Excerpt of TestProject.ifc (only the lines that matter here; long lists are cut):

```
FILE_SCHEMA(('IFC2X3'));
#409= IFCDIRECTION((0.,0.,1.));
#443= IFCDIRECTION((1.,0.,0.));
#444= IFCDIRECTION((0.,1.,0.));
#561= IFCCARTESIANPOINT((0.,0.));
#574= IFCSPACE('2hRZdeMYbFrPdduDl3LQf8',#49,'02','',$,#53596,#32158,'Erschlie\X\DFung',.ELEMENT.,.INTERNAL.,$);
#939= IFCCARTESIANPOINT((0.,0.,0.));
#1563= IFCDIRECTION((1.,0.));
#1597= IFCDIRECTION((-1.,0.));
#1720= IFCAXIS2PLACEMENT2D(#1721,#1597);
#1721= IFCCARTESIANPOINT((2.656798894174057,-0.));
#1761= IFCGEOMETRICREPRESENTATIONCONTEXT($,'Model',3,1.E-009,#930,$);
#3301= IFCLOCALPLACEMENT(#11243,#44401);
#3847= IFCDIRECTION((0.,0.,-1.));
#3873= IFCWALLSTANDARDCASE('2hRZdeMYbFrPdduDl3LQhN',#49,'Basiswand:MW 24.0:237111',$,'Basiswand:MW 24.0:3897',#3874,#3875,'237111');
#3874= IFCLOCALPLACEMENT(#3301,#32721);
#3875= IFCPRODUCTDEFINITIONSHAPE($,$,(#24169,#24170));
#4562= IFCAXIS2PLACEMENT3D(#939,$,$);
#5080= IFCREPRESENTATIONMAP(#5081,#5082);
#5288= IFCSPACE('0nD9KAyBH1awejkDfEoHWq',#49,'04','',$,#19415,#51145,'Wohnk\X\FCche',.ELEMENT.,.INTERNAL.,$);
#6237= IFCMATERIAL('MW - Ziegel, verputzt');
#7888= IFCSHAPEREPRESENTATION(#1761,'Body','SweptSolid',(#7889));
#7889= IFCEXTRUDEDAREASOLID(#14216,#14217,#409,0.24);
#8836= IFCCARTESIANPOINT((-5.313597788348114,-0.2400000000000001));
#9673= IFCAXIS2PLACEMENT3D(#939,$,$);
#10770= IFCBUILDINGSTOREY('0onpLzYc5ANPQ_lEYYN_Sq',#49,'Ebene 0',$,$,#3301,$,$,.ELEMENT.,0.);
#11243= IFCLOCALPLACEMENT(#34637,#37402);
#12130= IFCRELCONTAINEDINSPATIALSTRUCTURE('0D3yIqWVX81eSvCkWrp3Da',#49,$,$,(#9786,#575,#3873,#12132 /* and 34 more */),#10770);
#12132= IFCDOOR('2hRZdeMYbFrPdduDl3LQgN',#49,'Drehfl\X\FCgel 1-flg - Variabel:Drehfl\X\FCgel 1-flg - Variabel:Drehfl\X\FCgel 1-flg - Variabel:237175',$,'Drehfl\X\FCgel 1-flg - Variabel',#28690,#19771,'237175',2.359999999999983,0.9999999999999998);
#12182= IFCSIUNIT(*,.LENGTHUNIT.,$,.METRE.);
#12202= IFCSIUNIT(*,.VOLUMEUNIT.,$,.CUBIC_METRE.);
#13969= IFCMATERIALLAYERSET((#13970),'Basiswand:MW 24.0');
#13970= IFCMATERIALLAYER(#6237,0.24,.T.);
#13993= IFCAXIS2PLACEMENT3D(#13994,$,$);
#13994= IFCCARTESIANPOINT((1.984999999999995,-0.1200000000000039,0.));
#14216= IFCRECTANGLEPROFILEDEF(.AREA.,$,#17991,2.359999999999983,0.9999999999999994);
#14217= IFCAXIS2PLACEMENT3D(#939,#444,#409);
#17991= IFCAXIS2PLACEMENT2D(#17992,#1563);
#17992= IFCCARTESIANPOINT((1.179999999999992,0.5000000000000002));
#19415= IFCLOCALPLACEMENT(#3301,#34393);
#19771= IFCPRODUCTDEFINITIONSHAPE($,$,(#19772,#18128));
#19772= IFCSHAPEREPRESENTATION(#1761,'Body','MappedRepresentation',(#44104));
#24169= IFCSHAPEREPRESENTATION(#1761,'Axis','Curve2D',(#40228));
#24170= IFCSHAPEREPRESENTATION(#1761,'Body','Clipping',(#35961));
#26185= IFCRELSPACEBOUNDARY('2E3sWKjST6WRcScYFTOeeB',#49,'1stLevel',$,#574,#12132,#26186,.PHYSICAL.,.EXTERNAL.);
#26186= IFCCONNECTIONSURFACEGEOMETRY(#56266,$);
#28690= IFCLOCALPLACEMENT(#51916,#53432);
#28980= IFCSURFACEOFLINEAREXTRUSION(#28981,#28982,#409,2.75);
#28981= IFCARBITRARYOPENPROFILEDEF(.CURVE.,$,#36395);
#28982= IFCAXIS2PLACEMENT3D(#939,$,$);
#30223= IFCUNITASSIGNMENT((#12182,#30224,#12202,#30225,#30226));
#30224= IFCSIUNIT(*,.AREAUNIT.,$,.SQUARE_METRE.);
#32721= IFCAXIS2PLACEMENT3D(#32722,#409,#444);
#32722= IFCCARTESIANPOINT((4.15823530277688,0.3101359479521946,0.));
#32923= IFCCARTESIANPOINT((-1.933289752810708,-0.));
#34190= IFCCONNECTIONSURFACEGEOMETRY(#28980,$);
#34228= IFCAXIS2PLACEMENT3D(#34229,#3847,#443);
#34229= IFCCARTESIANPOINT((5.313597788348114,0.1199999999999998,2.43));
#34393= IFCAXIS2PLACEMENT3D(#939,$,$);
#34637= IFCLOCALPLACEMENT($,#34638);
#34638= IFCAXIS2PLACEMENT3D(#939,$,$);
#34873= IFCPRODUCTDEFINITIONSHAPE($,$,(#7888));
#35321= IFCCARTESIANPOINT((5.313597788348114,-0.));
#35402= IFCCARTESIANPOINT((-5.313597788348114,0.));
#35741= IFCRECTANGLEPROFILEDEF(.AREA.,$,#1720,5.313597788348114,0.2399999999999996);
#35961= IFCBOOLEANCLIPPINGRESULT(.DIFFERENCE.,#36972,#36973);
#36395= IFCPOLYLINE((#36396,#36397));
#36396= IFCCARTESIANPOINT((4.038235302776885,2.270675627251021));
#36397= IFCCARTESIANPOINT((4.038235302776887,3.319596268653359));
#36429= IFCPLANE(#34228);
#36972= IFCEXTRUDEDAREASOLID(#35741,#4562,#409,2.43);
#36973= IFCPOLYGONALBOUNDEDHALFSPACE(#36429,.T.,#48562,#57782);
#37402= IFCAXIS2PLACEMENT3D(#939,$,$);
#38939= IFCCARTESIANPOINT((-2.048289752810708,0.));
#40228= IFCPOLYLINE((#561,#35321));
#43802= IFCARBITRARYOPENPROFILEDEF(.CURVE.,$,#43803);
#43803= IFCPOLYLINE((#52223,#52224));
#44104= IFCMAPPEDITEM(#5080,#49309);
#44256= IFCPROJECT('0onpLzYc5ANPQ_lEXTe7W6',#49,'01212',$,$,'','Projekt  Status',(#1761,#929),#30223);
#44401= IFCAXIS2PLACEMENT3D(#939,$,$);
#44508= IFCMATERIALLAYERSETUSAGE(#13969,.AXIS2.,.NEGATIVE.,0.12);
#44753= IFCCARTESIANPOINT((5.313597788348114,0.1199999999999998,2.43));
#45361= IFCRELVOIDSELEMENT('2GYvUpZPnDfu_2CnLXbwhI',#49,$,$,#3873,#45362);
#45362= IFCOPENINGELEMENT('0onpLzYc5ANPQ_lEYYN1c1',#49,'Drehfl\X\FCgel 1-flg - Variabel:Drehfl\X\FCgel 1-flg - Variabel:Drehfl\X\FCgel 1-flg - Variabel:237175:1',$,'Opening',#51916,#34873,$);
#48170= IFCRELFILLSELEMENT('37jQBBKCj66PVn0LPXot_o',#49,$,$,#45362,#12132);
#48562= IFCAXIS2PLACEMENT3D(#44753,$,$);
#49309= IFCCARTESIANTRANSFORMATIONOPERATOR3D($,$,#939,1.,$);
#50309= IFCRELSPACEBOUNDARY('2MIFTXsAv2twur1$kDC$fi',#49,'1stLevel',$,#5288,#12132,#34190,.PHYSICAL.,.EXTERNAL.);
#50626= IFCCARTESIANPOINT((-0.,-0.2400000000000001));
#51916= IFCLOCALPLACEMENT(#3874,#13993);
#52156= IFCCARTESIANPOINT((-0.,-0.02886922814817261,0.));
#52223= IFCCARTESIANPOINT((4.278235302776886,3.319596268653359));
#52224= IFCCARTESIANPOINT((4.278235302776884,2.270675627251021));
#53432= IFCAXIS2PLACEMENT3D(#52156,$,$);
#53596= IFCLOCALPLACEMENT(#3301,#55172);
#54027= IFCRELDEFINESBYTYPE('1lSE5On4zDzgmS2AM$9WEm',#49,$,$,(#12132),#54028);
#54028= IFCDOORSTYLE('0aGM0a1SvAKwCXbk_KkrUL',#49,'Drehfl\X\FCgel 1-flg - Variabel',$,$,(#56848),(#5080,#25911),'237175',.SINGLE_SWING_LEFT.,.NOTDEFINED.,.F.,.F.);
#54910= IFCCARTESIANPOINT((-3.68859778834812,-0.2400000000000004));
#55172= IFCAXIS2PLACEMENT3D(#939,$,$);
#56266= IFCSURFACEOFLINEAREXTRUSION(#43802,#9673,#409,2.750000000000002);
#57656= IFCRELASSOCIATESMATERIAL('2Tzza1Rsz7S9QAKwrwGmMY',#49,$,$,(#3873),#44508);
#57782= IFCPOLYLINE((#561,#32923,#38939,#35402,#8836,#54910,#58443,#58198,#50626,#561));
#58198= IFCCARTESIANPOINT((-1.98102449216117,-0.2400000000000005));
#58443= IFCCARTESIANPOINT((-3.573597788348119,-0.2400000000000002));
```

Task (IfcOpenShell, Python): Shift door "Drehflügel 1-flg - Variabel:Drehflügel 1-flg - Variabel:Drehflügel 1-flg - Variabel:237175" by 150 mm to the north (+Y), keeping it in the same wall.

```python
import numpy as np
import ifcopenshell
import ifcopenshell.api.geometry
import ifcopenshell.util.placement
import ifcopenshell.util.unit

model = ifcopenshell.open("TestProject.ifc")
unit_scale = ifcopenshell.util.unit.calculate_unit_scale(model)

door = model.by_guid("2hRZdeMYbFrPdduDl3LQgN")
opening = door.FillsVoids[0].RelatingOpeningElement
wall = opening.VoidsElements[0].RelatingBuildingElement

wall_matrix = ifcopenshell.util.placement.get_local_placement(wall.ObjectPlacement)
shift = wall_matrix[:3, 0] * 0.15 / unit_scale
before = ifcopenshell.util.placement.get_local_placement(door.ObjectPlacement)[:3, 3].copy()

# The door is placed relative to its opening, so it follows when the opening moves.
matrix = ifcopenshell.util.placement.get_local_placement(opening.ObjectPlacement)
matrix[:3, 3] += shift
ifcopenshell.api.geometry.edit_object_placement(
    model, product=opening, matrix=matrix, is_si=False, should_transform_children=True
)

# Space boundary surfaces are stored in each space's coordinates; move them too.
for rel in door.ProvidesBoundaries:
    if not rel.ConnectionGeometry:
        continue
    surface = rel.ConnectionGeometry.SurfaceOnRelatingElement
    space_matrix = ifcopenshell.util.placement.get_local_placement(rel.RelatingSpace.ObjectPlacement)
    point = np.array(surface.Position.Location.Coordinates) + space_matrix[:3, :3].T @ shift
    surface.Position = model.createIfcAxis2Placement3D(
        model.createIfcCartesianPoint(point.tolist()), surface.Position.Axis, surface.Position.RefDirection
    )

after = ifcopenshell.util.placement.get_local_placement(door.ObjectPlacement)[:3, 3]
print("door moved by", (after - before).round(3) + 0.0)

model.write("TestProject_edited.ifc")
```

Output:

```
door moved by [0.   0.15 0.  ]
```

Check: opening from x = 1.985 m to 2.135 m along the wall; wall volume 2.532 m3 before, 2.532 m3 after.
